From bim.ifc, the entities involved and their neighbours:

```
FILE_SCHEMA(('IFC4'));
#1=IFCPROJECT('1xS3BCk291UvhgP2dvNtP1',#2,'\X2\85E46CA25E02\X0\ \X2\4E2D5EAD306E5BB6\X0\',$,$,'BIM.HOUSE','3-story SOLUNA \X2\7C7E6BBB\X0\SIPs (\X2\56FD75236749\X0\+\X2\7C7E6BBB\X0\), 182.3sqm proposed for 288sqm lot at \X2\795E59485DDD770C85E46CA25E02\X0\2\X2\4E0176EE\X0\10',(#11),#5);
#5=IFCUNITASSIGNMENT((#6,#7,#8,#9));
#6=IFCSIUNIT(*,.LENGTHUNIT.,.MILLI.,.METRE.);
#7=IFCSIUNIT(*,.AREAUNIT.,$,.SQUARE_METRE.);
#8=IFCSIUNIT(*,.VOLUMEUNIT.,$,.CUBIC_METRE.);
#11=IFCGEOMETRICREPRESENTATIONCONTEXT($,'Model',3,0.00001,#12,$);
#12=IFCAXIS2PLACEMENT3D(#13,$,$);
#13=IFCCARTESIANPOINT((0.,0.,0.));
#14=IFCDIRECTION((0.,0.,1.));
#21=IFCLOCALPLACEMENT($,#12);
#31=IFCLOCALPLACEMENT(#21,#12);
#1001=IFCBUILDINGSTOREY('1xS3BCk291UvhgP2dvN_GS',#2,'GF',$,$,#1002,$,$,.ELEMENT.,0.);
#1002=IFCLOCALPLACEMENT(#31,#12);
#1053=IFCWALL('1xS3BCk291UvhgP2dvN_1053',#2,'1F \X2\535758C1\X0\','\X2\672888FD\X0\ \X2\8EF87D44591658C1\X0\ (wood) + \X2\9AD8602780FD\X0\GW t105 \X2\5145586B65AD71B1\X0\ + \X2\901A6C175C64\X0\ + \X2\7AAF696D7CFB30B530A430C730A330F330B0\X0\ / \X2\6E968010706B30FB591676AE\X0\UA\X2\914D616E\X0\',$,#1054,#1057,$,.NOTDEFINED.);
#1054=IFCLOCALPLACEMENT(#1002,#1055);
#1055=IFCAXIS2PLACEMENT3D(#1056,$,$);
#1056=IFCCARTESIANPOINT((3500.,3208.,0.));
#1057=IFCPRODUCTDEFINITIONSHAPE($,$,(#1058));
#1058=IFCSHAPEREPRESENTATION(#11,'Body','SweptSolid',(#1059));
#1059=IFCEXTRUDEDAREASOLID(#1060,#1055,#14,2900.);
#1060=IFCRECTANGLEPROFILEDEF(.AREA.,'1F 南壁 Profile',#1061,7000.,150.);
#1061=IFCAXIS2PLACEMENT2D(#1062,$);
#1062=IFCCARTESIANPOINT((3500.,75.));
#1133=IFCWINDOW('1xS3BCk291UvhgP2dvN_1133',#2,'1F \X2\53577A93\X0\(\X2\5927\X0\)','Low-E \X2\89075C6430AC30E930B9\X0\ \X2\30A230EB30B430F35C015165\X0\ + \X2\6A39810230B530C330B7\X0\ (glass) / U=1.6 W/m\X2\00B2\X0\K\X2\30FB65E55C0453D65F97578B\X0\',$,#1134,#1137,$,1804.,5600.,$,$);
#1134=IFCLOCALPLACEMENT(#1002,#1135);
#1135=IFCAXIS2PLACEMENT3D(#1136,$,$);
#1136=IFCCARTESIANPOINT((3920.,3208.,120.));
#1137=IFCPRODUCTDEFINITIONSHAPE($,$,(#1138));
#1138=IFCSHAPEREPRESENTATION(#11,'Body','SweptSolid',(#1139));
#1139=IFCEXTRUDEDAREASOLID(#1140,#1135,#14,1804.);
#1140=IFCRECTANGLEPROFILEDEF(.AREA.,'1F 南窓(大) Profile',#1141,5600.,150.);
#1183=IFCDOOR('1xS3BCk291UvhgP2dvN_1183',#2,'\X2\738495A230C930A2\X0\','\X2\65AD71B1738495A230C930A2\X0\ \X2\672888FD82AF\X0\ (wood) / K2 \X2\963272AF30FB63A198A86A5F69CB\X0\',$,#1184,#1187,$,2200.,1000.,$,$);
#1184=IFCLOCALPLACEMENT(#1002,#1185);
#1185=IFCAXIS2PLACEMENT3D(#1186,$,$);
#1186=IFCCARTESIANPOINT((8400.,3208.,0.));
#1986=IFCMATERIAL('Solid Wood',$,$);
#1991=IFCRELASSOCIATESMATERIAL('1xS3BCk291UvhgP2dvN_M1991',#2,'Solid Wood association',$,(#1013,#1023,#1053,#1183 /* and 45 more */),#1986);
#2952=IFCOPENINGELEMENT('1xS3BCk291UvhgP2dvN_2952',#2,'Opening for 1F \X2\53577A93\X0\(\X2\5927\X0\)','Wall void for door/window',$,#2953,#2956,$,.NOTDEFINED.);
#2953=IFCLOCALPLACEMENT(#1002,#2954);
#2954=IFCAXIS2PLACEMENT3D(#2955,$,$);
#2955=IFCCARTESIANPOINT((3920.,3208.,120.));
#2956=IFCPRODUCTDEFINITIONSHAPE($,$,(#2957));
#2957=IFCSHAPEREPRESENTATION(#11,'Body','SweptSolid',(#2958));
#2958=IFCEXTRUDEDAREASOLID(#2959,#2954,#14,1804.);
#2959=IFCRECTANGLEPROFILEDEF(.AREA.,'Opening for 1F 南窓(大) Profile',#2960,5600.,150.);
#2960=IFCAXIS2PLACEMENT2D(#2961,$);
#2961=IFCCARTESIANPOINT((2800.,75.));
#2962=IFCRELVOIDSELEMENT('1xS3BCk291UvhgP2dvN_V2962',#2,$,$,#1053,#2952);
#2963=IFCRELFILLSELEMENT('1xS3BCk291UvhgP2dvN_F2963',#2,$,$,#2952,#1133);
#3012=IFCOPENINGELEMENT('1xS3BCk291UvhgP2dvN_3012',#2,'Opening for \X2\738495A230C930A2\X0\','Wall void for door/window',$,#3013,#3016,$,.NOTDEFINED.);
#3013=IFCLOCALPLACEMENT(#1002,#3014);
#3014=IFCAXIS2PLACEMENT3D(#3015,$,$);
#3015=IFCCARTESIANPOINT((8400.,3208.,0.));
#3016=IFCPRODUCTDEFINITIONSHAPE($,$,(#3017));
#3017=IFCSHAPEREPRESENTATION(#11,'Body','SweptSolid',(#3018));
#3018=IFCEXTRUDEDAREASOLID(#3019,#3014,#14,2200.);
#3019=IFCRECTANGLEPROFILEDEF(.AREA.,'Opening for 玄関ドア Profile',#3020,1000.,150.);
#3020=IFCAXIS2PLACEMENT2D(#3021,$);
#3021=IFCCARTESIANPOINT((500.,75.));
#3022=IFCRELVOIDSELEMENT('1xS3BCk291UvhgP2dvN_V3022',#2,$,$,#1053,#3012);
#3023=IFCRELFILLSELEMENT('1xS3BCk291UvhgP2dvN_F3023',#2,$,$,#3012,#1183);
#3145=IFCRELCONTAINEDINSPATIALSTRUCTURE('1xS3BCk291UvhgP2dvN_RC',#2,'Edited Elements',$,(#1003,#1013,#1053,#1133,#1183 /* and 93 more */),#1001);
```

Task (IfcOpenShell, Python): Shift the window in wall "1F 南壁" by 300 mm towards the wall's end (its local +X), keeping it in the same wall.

```python
import ifcopenshell
import ifcopenshell.api.geometry
import ifcopenshell.util.placement

model = ifcopenshell.open("bim.ifc")

window = model.by_guid("1xS3BCk291UvhgP2dvN_1133")
opening = window.FillsVoids[0].RelatingOpeningElement
wall = opening.VoidsElements[0].RelatingBuildingElement

wall_matrix = ifcopenshell.util.placement.get_local_placement(wall.ObjectPlacement)
shift = wall_matrix[:3, 0] * 300.0
before = ifcopenshell.util.placement.get_local_placement(window.ObjectPlacement)[:3, 3].copy()

# The window is not placed relative to its opening, so move both.
for product in (opening, window):
    matrix = ifcopenshell.util.placement.get_local_placement(product.ObjectPlacement)
    matrix[:3, 3] += shift
    ifcopenshell.api.geometry.edit_object_placement(model, product=product, matrix=matrix, is_si=False)

after = ifcopenshell.util.placement.get_local_placement(window.ObjectPlacement)[:3, 3]
print("window moved by", (after - before).round(3) + 0.0)

model.write("bim_rev.ifc")
```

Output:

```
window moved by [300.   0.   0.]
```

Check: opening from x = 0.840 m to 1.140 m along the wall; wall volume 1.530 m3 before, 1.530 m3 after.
